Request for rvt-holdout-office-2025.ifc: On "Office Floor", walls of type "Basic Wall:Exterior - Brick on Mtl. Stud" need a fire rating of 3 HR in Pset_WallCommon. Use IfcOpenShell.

First a look at what the model holds.

```python
import ifcopenshell
import ifcopenshell.util.element

model = ifcopenshell.open("rvt-holdout-office-2025.ifc")
print(model.schema)
storey = next(s for s in model.by_type("IfcBuildingStorey") if s.Name == "Office Floor")
walls = [e for e in ifcopenshell.util.element.get_decomposition(storey) if e.is_a("IfcWall")]
seen = {}
for e in walls:
    element_type = ifcopenshell.util.element.get_type(e)
    key = (element_type.Name if element_type != e and element_type else None, ifcopenshell.util.element.get_pset(e, "Pset_WallCommon", "FireRating"))
    seen[key] = seen.get(key, 0) + 1
for (name, value), count in sorted(seen.items(), key=str):
    print(count, "x", name, "|", value)
```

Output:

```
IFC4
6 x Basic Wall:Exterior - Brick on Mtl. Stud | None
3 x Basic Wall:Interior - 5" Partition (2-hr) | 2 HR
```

```python
import ifcopenshell
import ifcopenshell.api.pset
import ifcopenshell.util.element

model = ifcopenshell.open("rvt-holdout-office-2025.ifc")

storey = next(s for s in model.by_type("IfcBuildingStorey") if s.Name == "Office Floor")
walls = [e for e in ifcopenshell.util.element.get_decomposition(storey) if e.is_a("IfcWall")]

count = 0
for e in walls:
    element_type = ifcopenshell.util.element.get_type(e)
    if element_type in (None, e) or element_type.Name != "Basic Wall:Exterior - Brick on Mtl. Stud":
        continue
    # add_pset returns the element's existing set when there is one.
    pset = ifcopenshell.api.pset.add_pset(model, product=e, name="Pset_WallCommon")
    ifcopenshell.api.pset.edit_pset(model, pset=pset, properties={"FireRating": "3 HR"})
    count += 1

print(count, "walls updated")

model.write("rvt-holdout-office-2025_rev.ifc")
```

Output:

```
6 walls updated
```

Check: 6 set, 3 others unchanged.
